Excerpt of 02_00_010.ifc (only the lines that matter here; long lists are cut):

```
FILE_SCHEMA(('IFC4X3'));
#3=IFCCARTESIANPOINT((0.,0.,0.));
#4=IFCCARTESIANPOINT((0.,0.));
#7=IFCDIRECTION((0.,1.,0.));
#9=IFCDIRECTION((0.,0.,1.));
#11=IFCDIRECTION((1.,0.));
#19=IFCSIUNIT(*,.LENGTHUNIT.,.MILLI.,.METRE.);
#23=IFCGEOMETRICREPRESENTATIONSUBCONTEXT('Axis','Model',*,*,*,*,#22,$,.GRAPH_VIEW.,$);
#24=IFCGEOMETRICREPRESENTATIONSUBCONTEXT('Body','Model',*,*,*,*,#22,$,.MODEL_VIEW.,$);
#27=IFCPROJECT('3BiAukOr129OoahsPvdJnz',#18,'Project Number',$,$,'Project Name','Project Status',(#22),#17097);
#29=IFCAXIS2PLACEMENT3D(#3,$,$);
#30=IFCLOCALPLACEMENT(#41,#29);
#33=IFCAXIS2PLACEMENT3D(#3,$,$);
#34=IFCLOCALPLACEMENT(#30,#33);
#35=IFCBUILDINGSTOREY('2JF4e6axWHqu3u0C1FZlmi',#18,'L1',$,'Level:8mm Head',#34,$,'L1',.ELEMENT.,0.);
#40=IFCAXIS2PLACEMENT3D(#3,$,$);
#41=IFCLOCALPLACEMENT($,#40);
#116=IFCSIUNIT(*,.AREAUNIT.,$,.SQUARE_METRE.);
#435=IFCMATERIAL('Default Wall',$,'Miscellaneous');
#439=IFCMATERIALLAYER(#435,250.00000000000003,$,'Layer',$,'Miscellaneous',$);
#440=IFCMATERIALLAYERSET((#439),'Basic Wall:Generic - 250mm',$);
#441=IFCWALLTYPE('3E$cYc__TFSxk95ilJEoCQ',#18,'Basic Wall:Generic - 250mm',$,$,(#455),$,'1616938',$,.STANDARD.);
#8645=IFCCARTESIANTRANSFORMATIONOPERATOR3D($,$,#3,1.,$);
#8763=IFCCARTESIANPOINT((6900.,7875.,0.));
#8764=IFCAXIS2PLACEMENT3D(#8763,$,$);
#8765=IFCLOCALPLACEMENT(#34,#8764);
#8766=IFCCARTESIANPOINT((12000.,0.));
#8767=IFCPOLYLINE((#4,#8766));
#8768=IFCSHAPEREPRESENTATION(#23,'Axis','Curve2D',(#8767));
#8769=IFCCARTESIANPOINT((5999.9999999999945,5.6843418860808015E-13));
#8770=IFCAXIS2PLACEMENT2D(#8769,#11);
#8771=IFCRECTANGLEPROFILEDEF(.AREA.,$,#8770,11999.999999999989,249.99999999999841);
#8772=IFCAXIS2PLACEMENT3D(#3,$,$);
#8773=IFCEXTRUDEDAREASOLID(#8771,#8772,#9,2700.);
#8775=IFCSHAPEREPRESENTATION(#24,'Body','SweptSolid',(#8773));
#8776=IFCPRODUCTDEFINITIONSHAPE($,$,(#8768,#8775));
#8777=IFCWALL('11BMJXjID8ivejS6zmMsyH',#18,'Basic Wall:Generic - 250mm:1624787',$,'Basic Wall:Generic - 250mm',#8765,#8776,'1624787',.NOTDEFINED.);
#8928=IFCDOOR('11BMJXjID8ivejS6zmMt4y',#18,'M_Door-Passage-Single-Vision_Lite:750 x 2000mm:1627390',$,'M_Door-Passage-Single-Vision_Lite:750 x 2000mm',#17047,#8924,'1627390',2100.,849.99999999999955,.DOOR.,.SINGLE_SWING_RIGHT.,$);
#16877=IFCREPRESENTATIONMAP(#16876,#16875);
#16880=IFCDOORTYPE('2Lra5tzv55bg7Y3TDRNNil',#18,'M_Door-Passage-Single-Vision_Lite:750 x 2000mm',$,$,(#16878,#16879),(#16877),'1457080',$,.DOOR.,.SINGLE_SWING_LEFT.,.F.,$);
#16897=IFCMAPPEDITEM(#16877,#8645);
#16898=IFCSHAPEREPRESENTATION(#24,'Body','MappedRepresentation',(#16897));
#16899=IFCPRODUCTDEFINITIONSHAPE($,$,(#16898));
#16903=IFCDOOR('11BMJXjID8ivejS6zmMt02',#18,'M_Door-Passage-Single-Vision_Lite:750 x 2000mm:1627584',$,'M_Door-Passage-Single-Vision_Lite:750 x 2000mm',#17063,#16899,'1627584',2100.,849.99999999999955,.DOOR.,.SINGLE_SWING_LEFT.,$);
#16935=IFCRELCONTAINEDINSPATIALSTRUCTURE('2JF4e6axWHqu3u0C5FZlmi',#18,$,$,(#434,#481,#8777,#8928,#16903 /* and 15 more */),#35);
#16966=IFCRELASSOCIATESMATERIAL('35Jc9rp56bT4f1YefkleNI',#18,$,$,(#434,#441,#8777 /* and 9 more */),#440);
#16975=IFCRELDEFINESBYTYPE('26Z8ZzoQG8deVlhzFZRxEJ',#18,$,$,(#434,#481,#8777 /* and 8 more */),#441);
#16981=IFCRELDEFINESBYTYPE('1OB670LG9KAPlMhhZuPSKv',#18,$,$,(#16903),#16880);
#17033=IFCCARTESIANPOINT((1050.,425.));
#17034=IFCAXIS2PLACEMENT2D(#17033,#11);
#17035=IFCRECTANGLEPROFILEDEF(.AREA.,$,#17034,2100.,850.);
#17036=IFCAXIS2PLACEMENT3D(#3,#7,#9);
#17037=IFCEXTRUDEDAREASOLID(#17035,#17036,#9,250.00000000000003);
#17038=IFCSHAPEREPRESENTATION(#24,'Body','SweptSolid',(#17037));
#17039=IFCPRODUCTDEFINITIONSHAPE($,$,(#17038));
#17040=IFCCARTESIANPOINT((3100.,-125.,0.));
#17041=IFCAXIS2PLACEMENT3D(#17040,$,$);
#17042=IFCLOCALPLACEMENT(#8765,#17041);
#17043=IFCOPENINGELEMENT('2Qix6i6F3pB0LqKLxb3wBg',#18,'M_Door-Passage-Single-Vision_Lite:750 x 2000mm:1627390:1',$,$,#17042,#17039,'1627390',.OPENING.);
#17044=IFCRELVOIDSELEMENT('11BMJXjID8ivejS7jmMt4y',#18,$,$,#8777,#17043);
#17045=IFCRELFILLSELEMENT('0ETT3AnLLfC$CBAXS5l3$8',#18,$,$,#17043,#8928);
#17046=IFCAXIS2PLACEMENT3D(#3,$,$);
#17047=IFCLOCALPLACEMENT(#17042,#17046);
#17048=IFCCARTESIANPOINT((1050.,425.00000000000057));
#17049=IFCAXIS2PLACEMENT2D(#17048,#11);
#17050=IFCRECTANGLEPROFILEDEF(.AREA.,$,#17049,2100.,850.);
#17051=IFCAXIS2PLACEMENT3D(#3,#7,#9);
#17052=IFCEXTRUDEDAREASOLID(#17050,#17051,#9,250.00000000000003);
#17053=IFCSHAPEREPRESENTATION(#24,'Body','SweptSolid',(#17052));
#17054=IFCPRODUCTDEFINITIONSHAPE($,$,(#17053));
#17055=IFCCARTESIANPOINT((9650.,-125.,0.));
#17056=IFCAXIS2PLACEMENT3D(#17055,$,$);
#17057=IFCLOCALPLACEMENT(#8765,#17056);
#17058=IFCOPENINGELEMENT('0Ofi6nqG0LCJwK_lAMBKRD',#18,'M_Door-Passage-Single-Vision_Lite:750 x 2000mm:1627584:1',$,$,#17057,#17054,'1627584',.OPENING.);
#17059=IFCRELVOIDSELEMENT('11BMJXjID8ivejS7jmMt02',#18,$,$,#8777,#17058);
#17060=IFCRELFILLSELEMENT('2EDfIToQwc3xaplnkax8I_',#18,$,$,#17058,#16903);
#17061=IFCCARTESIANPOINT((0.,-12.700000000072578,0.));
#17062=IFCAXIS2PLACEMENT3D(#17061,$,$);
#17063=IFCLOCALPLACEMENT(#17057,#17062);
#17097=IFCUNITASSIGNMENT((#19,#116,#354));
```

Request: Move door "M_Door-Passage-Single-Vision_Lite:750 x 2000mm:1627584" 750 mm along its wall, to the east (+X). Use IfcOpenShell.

```python
import ifcopenshell
import ifcopenshell.api.geometry
import ifcopenshell.util.placement

model = ifcopenshell.open("02_00_010.ifc")

door = model.by_guid("11BMJXjID8ivejS6zmMt02")
opening = door.FillsVoids[0].RelatingOpeningElement
wall = opening.VoidsElements[0].RelatingBuildingElement

wall_matrix = ifcopenshell.util.placement.get_local_placement(wall.ObjectPlacement)
shift = wall_matrix[:3, 0] * 750.0
before = ifcopenshell.util.placement.get_local_placement(door.ObjectPlacement)[:3, 3].copy()

# The door is placed relative to its opening, so it follows when the opening moves.
matrix = ifcopenshell.util.placement.get_local_placement(opening.ObjectPlacement)
matrix[:3, 3] += shift
ifcopenshell.api.geometry.edit_object_placement(
    model, product=opening, matrix=matrix, is_si=False, should_transform_children=True
)

after = ifcopenshell.util.placement.get_local_placement(door.ObjectPlacement)[:3, 3]
print("door moved by", (after - before).round(3) + 0.0)

model.write("02_00_010_rev.ifc")
```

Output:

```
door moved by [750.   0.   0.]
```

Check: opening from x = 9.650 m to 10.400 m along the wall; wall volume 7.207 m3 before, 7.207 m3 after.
